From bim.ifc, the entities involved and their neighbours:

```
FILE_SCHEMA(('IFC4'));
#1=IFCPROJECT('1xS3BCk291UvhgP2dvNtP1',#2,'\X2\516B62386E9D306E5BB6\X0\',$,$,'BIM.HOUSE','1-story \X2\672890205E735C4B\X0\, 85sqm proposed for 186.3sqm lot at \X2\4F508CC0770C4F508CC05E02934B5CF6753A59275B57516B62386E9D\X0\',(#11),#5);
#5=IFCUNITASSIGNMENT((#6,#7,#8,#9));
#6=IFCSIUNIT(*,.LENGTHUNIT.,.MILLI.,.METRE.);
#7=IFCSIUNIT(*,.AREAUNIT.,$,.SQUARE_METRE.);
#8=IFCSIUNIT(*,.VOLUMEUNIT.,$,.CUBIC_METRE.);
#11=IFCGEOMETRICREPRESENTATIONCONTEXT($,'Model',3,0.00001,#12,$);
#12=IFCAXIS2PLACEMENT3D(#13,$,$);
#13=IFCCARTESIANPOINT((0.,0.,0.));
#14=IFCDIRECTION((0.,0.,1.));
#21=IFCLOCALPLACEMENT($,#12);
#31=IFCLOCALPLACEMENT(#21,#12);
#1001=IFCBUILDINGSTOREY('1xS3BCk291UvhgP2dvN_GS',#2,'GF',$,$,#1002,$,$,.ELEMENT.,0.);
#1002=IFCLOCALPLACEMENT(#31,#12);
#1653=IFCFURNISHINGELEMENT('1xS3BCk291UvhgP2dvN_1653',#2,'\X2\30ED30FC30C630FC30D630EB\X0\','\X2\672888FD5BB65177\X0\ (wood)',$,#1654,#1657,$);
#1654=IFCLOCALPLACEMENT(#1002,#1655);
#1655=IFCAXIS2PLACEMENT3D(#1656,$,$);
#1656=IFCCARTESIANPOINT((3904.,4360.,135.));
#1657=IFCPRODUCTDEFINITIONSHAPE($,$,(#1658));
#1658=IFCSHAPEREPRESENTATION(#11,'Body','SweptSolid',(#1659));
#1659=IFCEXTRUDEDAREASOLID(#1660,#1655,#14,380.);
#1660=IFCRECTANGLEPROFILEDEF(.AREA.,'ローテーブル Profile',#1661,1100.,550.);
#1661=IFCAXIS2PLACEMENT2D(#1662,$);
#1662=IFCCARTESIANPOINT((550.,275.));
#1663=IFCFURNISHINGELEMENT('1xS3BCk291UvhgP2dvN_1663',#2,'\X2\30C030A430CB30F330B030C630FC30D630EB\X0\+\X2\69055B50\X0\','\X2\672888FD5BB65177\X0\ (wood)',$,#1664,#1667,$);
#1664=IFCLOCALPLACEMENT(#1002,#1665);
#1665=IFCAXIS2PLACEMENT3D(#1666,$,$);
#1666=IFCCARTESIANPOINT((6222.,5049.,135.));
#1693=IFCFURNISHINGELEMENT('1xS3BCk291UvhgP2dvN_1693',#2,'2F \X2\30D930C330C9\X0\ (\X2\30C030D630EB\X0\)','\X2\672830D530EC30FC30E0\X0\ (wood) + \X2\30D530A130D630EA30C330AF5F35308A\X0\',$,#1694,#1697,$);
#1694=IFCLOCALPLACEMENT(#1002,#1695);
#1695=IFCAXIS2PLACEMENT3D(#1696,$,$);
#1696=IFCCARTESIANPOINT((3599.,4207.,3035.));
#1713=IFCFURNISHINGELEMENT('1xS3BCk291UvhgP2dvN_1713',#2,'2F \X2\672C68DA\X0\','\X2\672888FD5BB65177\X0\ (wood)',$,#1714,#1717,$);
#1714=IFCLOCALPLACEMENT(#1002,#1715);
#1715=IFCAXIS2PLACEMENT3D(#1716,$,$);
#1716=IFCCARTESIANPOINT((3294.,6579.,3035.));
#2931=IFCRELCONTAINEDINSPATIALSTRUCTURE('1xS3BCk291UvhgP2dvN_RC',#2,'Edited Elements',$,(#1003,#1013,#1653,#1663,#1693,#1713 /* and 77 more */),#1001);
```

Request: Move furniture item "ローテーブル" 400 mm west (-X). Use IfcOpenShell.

```python
import ifcopenshell
import ifcopenshell.api.geometry
import ifcopenshell.util.placement
import ifcopenshell.util.unit

model = ifcopenshell.open("bim.ifc")
unit_scale = ifcopenshell.util.unit.calculate_unit_scale(model)

item = model.by_guid("1xS3BCk291UvhgP2dvN_1653")
matrix = ifcopenshell.util.placement.get_local_placement(item.ObjectPlacement)
matrix[0, 3] -= 0.4 / unit_scale
ifcopenshell.api.geometry.edit_object_placement(model, product=item, matrix=matrix, is_si=False)

print(ifcopenshell.util.placement.get_local_placement(item.ObjectPlacement).round(3) + 0.0)

model.write("bim_updated.ifc")
```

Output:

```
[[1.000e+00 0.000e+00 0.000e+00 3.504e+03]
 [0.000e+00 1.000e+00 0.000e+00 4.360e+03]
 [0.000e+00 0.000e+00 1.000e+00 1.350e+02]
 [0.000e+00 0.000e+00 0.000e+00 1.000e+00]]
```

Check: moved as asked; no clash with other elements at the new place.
